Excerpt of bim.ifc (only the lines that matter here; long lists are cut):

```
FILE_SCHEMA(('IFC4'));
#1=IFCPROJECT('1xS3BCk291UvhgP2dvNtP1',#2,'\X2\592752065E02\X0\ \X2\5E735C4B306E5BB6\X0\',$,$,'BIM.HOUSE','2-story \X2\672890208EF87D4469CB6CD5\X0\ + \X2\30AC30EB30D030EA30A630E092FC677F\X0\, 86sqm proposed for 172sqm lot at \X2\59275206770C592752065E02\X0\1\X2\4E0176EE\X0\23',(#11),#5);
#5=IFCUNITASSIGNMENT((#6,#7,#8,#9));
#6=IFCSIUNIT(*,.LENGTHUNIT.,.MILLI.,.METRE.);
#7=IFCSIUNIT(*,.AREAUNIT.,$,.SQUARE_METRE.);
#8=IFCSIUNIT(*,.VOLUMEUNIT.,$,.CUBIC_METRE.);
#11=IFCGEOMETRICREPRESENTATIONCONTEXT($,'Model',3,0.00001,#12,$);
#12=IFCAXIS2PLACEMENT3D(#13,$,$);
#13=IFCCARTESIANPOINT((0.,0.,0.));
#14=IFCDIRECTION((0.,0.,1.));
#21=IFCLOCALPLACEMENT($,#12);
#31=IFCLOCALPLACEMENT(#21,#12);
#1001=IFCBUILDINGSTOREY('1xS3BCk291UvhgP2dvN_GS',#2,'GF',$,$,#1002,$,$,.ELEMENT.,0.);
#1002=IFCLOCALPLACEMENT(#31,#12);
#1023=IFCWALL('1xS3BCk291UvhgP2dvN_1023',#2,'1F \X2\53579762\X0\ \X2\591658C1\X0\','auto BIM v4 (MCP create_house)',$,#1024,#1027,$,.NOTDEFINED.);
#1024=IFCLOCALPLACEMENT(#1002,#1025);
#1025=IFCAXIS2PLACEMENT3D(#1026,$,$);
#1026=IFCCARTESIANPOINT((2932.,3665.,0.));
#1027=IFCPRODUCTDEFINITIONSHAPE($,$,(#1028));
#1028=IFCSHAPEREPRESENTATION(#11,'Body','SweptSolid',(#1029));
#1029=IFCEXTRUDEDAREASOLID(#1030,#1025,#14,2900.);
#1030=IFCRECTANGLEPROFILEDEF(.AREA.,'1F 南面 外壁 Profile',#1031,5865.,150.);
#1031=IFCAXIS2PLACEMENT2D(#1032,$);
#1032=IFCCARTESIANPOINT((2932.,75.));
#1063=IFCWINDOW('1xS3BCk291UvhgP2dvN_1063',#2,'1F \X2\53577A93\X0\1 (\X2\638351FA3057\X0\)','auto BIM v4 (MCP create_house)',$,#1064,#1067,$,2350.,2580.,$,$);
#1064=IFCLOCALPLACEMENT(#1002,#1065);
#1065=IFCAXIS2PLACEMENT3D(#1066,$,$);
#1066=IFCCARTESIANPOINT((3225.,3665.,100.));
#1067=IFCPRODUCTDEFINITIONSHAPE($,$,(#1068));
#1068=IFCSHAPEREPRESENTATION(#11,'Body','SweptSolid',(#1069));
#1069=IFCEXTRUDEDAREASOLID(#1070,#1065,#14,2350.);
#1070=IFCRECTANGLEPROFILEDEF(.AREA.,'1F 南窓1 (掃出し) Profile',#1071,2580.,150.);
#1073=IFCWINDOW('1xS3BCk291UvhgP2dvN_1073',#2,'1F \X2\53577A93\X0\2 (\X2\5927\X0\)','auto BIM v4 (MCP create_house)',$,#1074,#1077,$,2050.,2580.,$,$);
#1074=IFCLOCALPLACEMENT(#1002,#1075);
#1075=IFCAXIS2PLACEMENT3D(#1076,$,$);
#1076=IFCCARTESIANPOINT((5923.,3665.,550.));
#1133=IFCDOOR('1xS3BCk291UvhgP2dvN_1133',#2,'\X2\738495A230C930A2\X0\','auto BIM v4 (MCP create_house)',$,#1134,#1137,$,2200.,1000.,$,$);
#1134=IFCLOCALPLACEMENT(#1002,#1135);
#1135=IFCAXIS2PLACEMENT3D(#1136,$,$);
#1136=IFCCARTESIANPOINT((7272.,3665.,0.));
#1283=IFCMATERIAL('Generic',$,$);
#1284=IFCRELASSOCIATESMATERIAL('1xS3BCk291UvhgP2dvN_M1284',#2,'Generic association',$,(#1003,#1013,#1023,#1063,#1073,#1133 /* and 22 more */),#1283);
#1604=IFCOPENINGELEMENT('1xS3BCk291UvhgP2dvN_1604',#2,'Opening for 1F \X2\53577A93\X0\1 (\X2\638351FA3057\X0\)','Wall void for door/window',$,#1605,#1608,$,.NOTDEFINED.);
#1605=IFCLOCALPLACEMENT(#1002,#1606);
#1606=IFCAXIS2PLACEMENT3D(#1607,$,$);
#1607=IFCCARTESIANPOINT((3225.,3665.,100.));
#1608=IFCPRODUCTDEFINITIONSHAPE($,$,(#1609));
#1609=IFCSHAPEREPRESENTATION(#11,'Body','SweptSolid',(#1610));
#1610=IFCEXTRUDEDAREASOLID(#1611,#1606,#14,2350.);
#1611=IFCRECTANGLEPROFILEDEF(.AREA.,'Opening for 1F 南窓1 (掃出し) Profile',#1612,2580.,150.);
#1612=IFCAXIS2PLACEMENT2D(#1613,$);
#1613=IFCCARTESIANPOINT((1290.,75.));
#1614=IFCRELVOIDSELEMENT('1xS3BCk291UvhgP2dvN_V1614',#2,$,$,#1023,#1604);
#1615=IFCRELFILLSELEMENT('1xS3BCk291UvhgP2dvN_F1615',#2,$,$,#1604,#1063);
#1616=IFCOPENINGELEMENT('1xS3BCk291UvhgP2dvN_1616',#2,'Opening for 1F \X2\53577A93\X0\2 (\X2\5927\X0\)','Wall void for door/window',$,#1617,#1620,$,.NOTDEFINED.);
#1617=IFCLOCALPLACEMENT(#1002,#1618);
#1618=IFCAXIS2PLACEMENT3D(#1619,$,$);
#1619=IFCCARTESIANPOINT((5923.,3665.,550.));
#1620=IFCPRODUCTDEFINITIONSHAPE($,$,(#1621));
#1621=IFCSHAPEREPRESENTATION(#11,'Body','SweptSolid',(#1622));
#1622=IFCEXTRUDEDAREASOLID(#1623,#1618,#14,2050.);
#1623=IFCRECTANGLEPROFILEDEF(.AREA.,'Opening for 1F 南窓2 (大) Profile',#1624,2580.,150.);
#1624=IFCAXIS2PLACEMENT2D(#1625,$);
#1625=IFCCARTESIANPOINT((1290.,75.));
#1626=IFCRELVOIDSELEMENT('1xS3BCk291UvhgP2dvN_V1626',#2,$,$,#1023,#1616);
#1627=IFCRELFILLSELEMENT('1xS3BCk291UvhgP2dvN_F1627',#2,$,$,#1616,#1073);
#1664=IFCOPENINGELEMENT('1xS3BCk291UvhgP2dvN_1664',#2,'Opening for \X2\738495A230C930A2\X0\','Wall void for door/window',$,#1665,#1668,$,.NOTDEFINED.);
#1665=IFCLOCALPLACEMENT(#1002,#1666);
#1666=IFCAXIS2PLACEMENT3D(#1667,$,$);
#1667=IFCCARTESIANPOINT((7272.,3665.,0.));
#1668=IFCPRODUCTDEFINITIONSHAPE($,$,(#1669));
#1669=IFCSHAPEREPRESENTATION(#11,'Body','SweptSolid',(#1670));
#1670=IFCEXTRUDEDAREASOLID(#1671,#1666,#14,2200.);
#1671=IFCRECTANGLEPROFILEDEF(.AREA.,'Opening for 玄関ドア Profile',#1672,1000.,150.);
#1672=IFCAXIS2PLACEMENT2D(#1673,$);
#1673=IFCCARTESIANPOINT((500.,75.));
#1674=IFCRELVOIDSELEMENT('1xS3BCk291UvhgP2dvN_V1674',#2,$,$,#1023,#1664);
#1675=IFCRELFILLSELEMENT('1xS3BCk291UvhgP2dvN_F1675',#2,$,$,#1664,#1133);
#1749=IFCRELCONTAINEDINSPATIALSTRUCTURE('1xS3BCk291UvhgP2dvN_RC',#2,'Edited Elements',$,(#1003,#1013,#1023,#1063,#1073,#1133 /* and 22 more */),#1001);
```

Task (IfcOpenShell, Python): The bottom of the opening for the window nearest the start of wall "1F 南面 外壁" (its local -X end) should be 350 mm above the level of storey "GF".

```python
import numpy as np
import ifcopenshell
import ifcopenshell.api.geometry
import ifcopenshell.geom
import ifcopenshell.util.element
import ifcopenshell.util.placement
import ifcopenshell.util.shape
import ifcopenshell.util.unit

model = ifcopenshell.open("bim.ifc")
unit_scale = ifcopenshell.util.unit.calculate_unit_scale(model)

window = model.by_id(1063)
opening = window.FillsVoids[0].RelatingOpeningElement
storey = ifcopenshell.util.element.get_container(window, ifc_class="IfcBuildingStorey")
level = ifcopenshell.util.placement.get_local_placement(storey.ObjectPlacement)[2, 3]

# The opening's origin need not be at the sill, so measure its lowest point.
shape = ifcopenshell.geom.create_shape(ifcopenshell.geom.settings(), opening)
bottom = ifcopenshell.util.shape.get_shape_bottom_elevation(shape, shape.geometry) / unit_scale
dz = level + 350.0 - bottom

shift = np.array([0.0, 0.0, dz])
# The window is not placed relative to its opening, so move both.
for product in (opening, window):
    matrix = ifcopenshell.util.placement.get_local_placement(product.ObjectPlacement)
    matrix[:3, 3] += shift
    ifcopenshell.api.geometry.edit_object_placement(model, product=product, matrix=matrix, is_si=False)

print(f"moved by {dz * unit_scale:+.3f} m")

model.write("bim_rev.ifc")
```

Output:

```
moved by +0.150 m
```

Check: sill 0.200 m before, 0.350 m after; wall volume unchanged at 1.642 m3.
